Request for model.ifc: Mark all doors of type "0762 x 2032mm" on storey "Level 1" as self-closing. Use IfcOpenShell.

First a look at what the model holds.

```python
import ifcopenshell
import ifcopenshell.util.element

model = ifcopenshell.open("model.ifc")
print(model.schema)
storey = next(s for s in model.by_type("IfcBuildingStorey") if s.Name == "Level 1")
doors = [e for e in ifcopenshell.util.element.get_decomposition(storey) if e.is_a("IfcDoor")]
seen = {}
for e in doors:
    element_type = ifcopenshell.util.element.get_type(e)
    key = (element_type.Name if element_type != e and element_type else None, ifcopenshell.util.element.get_pset(e, "Pset_DoorCommon", "SelfClosing"))
    seen[key] = seen.get(key, 0) + 1
for (name, value), count in sorted(seen.items(), key=str):
    print(count, "x", name, "|", value)
```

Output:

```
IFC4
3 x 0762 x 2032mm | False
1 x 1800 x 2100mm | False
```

```python
import ifcopenshell
import ifcopenshell.api.pset
import ifcopenshell.util.element

model = ifcopenshell.open("model.ifc")

storey = next(s for s in model.by_type("IfcBuildingStorey") if s.Name == "Level 1")
doors = [e for e in ifcopenshell.util.element.get_decomposition(storey) if e.is_a("IfcDoor")]

count = 0
for e in doors:
    element_type = ifcopenshell.util.element.get_type(e)
    if element_type in (None, e) or element_type.Name != "0762 x 2032mm":
        continue
    # add_pset returns the element's existing set when there is one.
    pset = ifcopenshell.api.pset.add_pset(model, product=e, name="Pset_DoorCommon")
    ifcopenshell.api.pset.edit_pset(model, pset=pset, properties={"SelfClosing": True})
    count += 1

print(count, "doors updated")

model.write("model_updated.ifc")
```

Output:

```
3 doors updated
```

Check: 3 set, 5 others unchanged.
